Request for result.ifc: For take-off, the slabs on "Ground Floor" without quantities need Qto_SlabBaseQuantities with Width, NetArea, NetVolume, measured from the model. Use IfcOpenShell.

First a look at what the model holds.

```python
import ifcopenshell
import ifcopenshell.util.element
import ifcopenshell.util.unit

model = ifcopenshell.open("result.ifc")
print(model.schema)
for unit_type in ("LENGTHUNIT", "AREAUNIT", "VOLUMEUNIT"):
    print(unit_type, ifcopenshell.util.unit.calculate_unit_scale(model, unit_type))
storey = next(s for s in model.by_type("IfcBuildingStorey") if s.Name == "Ground Floor")
slabs = [e for e in ifcopenshell.util.element.get_decomposition(storey) if e.is_a("IfcSlab")]
for e in sorted(slabs, key=lambda e: e.id()):
    print(e.id(), e.is_a(), e.Name, list(ifcopenshell.util.element.get_psets(e, qtos_only=True)), sep=" | ")
```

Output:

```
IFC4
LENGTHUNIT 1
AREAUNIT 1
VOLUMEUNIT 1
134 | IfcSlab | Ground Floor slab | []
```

```python
import ifcopenshell
import ifcopenshell.api.pset
import ifcopenshell.geom
import ifcopenshell.util.element
import ifcopenshell.util.shape
import ifcopenshell.util.unit

model = ifcopenshell.open("result.ifc")
unit_scale = ifcopenshell.util.unit.calculate_unit_scale(model)
area_scale = ifcopenshell.util.unit.calculate_unit_scale(model, "AREAUNIT")
volume_scale = ifcopenshell.util.unit.calculate_unit_scale(model, "VOLUMEUNIT")
settings = ifcopenshell.geom.settings()

storey = next(s for s in model.by_type("IfcBuildingStorey") if s.Name == "Ground Floor")
slabs = [e for e in ifcopenshell.util.element.get_decomposition(storey) if e.is_a("IfcSlab")]

for e in sorted(slabs, key=lambda e: e.id()):
    if ifcopenshell.util.element.get_psets(e, qtos_only=True, should_inherit=False):
        continue
    # Geometry comes back in metres, in the element's own axes.
    shape = ifcopenshell.geom.create_shape(settings, e)
    values = {
        "Width": ifcopenshell.util.shape.get_z(shape.geometry) / unit_scale,
        "NetArea": ifcopenshell.util.shape.get_footprint_area(shape.geometry) / area_scale,
        "NetVolume": ifcopenshell.util.shape.get_volume(shape.geometry) / volume_scale,
    }
    qto = ifcopenshell.api.pset.add_qto(model, product=e, name="Qto_SlabBaseQuantities")
    ifcopenshell.api.pset.edit_qto(model, qto=qto, properties=values)
    print(e.id(), {k: round(v, 3) for k, v in values.items()})

model.write("result-out.ifc")
```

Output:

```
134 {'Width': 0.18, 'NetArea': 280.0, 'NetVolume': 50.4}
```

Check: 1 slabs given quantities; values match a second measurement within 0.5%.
